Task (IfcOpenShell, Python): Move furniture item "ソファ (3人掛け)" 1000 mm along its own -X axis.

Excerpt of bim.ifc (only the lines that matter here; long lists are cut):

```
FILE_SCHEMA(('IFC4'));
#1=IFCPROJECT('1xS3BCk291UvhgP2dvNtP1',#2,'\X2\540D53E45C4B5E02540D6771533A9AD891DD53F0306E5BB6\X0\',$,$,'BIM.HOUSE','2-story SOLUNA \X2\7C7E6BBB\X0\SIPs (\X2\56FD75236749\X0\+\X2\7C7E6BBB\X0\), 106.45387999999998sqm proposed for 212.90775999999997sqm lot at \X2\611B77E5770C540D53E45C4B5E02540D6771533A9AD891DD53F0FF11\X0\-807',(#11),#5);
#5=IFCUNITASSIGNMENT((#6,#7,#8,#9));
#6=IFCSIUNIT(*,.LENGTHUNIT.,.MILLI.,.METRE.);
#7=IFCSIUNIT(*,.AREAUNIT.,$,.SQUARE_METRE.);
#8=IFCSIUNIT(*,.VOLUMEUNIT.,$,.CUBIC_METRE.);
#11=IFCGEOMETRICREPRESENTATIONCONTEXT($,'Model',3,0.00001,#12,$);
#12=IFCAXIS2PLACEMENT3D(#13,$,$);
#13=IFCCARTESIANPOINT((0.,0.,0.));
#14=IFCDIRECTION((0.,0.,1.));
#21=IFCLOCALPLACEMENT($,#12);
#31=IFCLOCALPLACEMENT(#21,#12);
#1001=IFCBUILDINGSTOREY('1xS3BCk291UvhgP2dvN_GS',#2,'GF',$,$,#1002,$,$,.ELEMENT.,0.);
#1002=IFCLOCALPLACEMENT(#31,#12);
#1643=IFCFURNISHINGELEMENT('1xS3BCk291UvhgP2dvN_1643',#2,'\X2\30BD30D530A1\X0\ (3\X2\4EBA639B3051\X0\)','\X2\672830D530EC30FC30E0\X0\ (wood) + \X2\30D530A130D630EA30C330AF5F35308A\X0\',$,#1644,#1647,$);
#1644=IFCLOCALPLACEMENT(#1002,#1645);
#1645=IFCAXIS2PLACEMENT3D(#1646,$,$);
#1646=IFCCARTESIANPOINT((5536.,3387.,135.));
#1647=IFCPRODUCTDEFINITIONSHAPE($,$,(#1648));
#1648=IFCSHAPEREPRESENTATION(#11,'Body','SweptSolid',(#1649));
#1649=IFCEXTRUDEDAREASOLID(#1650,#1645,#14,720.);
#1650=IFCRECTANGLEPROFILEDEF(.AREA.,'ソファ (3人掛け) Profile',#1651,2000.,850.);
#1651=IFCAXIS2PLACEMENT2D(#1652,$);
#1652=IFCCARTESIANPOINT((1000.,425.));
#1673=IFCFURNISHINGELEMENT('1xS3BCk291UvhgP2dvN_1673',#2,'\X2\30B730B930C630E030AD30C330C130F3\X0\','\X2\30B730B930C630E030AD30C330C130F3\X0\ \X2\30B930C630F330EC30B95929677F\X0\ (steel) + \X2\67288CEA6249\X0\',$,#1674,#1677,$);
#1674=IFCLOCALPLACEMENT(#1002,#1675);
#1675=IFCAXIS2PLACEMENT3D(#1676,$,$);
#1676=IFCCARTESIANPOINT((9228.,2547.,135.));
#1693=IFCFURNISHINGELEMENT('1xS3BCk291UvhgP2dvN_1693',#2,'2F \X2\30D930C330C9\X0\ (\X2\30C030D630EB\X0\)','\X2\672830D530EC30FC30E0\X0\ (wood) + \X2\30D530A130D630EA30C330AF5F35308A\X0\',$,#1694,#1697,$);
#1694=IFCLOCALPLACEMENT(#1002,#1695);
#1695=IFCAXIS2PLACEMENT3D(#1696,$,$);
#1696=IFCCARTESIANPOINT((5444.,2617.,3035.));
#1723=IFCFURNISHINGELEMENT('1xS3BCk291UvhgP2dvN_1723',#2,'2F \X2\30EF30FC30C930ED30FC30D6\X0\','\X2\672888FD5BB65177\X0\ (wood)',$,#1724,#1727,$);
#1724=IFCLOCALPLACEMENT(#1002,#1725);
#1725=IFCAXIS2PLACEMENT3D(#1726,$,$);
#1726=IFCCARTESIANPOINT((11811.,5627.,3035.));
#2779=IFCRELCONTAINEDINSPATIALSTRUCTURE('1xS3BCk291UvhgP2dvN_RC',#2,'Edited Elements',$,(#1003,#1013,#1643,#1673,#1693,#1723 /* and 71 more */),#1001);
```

```python
import ifcopenshell
import ifcopenshell.api.geometry
import ifcopenshell.util.placement

model = ifcopenshell.open("bim.ifc")

item = model.by_guid("1xS3BCk291UvhgP2dvN_1643")
matrix = ifcopenshell.util.placement.get_local_placement(item.ObjectPlacement)
matrix[:3, 3] -= matrix[:3, 0] * 1000.0
ifcopenshell.api.geometry.edit_object_placement(model, product=item, matrix=matrix, is_si=False)

print(ifcopenshell.util.placement.get_local_placement(item.ObjectPlacement).round(3) + 0.0)

model.write("bim_rev.ifc")
```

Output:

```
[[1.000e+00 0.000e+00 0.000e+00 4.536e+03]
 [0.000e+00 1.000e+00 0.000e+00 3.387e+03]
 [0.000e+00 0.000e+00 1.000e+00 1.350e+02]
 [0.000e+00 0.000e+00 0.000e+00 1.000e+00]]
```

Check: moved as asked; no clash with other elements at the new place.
